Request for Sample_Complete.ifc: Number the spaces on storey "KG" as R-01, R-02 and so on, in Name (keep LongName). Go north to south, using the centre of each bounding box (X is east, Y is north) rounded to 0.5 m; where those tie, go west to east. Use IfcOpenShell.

First a look at what the model holds.

```python
import ifcopenshell
import ifcopenshell.util.element
import ifcopenshell.util.placement

model = ifcopenshell.open("Sample_Complete.ifc")
print(model.schema)
storey = next(s for s in model.by_type("IfcBuildingStorey") if s.Name == "KG")
spaces = [e for e in ifcopenshell.util.element.get_decomposition(storey) if e.is_a("IfcSpace")]
for e in sorted(spaces, key=lambda e: e.id()):
    origin = ifcopenshell.util.placement.get_local_placement(e.ObjectPlacement)[:3, 3]
    print(e.id(), e.Name, e.LongName, origin.round(2) + 0.0, sep=" | ")
```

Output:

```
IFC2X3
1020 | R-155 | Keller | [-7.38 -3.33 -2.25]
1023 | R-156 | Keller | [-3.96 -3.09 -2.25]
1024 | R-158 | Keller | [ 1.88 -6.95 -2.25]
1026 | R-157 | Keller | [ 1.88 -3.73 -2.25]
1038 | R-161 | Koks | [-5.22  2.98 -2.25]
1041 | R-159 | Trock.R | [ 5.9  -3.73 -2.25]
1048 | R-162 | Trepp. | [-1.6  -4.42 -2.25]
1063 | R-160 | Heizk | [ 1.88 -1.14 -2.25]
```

```python
import ifcopenshell
import ifcopenshell.geom
import ifcopenshell.util.element
import ifcopenshell.util.shape

model = ifcopenshell.open("Sample_Complete.ifc")
settings = ifcopenshell.geom.settings()
settings.set("use-world-coords", True)


def centre(element):
    shape = ifcopenshell.geom.create_shape(settings, element)
    return ifcopenshell.util.shape.get_bbox_centroid(shape.geometry)


storey = next(s for s in model.by_type("IfcBuildingStorey") if s.Name == "KG")
spaces = [e for e in ifcopenshell.util.element.get_decomposition(storey) if e.is_a("IfcSpace")]

# Insertion points can sit at a corner or the storey origin, so sort by the geometry (in metres).
centres = {e: centre(e) for e in spaces}
spaces.sort(key=lambda e: (-round(centres[e][1] / 0.5), centres[e][0]))

for i, e in enumerate(spaces, start=1):
    number = f"R-{i:02d}"
    e.Name = number
    print(e.id(), number)

model.write("Sample_Complete_edited.ifc")
```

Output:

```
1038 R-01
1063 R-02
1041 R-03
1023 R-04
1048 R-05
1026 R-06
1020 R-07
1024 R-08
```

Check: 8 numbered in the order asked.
